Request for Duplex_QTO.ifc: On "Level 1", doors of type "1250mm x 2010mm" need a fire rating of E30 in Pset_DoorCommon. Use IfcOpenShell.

First a look at what the model holds.

```python
import ifcopenshell
import ifcopenshell.util.element

model = ifcopenshell.open("Duplex_QTO.ifc")
print(model.schema)
storey = next(s for s in model.by_type("IfcBuildingStorey") if s.Name == "Level 1")
doors = [e for e in ifcopenshell.util.element.get_decomposition(storey) if e.is_a("IfcDoor")]
seen = {}
for e in doors:
    element_type = ifcopenshell.util.element.get_type(e)
    key = (element_type.Name if element_type != e and element_type else None, ifcopenshell.util.element.get_pset(e, "Pset_DoorCommon", "FireRating"))
    seen[key] = seen.get(key, 0) + 1
for (name, value), count in sorted(seen.items(), key=str):
    print(count, "x", name, "|", value)
```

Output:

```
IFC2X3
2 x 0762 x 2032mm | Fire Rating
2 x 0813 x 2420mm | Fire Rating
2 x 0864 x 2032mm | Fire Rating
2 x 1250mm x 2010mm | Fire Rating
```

```python
import ifcopenshell
import ifcopenshell.api.pset
import ifcopenshell.util.element

model = ifcopenshell.open("Duplex_QTO.ifc")

storey = next(s for s in model.by_type("IfcBuildingStorey") if s.Name == "Level 1")
doors = [e for e in ifcopenshell.util.element.get_decomposition(storey) if e.is_a("IfcDoor")]

count = 0
for e in doors:
    element_type = ifcopenshell.util.element.get_type(e)
    if element_type in (None, e) or element_type.Name != "1250mm x 2010mm":
        continue
    # add_pset returns the element's existing set when there is one.
    pset = ifcopenshell.api.pset.add_pset(model, product=e, name="Pset_DoorCommon")
    ifcopenshell.api.pset.edit_pset(model, pset=pset, properties={"FireRating": "E30"})
    count += 1

print(count, "doors updated")

model.write("Duplex_QTO_rev.ifc")
```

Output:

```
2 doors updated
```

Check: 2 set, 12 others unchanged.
